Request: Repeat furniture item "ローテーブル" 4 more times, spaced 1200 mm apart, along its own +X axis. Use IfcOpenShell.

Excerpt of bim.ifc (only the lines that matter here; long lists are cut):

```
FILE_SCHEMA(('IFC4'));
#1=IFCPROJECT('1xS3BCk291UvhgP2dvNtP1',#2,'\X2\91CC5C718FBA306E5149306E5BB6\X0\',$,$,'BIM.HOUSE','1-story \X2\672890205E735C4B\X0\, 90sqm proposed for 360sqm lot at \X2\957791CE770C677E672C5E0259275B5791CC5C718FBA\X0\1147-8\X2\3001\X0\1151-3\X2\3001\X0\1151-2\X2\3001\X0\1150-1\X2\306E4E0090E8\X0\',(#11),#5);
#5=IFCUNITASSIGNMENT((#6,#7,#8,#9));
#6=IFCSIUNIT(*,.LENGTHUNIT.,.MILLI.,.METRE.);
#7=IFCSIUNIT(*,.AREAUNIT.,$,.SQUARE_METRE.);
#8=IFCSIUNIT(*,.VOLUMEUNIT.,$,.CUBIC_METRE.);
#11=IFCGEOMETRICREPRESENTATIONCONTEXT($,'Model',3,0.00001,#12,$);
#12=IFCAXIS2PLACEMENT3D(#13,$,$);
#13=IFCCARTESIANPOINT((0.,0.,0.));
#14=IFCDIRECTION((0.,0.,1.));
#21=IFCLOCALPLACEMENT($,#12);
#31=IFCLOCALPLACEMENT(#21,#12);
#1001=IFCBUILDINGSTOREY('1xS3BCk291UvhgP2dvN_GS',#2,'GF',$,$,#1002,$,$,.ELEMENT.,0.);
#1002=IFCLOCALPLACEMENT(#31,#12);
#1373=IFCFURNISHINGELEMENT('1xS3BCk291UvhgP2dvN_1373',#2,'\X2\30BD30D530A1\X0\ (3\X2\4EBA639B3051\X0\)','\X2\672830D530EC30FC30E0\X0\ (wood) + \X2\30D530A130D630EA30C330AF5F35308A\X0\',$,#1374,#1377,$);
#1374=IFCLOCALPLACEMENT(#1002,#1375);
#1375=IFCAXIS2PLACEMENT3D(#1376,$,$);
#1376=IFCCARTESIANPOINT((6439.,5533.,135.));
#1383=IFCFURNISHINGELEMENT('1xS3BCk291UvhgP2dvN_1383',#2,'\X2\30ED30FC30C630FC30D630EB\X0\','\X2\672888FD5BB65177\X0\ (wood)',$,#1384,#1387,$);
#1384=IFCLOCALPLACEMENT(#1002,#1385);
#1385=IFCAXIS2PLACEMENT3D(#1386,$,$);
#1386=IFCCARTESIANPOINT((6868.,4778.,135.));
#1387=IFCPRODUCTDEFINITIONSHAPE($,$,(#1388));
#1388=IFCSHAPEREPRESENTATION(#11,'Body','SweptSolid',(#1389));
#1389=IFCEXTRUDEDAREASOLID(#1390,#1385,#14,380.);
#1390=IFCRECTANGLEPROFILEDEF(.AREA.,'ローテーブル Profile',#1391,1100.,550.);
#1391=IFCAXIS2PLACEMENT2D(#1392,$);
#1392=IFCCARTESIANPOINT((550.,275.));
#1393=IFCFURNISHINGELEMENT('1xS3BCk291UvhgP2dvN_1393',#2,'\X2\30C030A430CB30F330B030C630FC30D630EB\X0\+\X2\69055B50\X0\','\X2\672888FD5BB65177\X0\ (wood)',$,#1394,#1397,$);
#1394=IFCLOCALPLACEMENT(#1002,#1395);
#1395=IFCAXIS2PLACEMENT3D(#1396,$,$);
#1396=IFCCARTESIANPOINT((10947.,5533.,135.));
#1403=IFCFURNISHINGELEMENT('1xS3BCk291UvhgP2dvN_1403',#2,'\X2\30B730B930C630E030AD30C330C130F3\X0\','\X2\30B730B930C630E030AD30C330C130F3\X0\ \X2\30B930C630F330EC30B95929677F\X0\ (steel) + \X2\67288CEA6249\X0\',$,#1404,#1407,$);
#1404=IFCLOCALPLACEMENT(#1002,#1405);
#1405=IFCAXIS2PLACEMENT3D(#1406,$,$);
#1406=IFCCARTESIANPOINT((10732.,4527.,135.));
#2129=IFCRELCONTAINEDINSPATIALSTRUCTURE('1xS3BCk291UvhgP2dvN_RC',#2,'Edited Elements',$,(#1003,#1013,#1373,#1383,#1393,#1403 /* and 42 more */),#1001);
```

```python
import ifcopenshell
import ifcopenshell.api.geometry
import ifcopenshell.api.root
import ifcopenshell.util.element
import ifcopenshell.util.placement
import ifcopenshell.util.unit

model = ifcopenshell.open("bim.ifc")
unit_scale = ifcopenshell.util.unit.calculate_unit_scale(model)


def reuse_history(source, copy):
    """copy_class also copies each property set's owner history, people and application; keep the originals."""
    for rel in copy.IsDefinedBy:
        if rel.is_a("IfcRelDefinesByProperties") and (history := rel.RelatingPropertyDefinition.OwnerHistory):
            rel.RelatingPropertyDefinition.OwnerHistory = source.OwnerHistory
            ifcopenshell.util.element.remove_deep2(model, history)


source = model.by_guid("1xS3BCk291UvhgP2dvN_1383")
base = ifcopenshell.util.placement.get_local_placement(source.ObjectPlacement)
step = base[:3, 0] * 1.2 / unit_scale

for i in range(1, 5):
    copy = ifcopenshell.api.root.copy_class(model, product=source)
    copy.Representation = ifcopenshell.util.element.copy_deep(
        model, source.Representation, exclude=["IfcGeometricRepresentationContext", "IfcRepresentationMap"]
    )
    reuse_history(source, copy)
    matrix = base.copy()
    matrix[:3, 3] += i * step
    print("added at", matrix[:3, 3].round(3) + 0.0)
    ifcopenshell.api.geometry.edit_object_placement(model, product=copy, matrix=matrix, is_si=False)

model.write("bim-out.ifc")
```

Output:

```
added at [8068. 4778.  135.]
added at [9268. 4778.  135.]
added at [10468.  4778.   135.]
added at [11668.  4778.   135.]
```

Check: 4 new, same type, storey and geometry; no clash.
